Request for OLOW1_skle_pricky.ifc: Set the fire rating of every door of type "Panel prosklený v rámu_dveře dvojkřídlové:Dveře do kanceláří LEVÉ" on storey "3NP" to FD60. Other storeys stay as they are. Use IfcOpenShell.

First a look at what the model holds.

```python
import ifcopenshell
import ifcopenshell.util.element

model = ifcopenshell.open("OLOW1_skle_pricky.ifc")
print(model.schema)
storey = next(s for s in model.by_type("IfcBuildingStorey") if s.Name == "3NP")
doors = [e for e in ifcopenshell.util.element.get_decomposition(storey) if e.is_a("IfcDoor")]
seen = {}
for e in doors:
    element_type = ifcopenshell.util.element.get_type(e)
    key = (element_type.Name if element_type != e and element_type else None, ifcopenshell.util.element.get_pset(e, "Pset_DoorCommon", "FireRating"))
    seen[key] = seen.get(key, 0) + 1
for (name, value), count in sorted(seen.items(), key=str):
    print(count, "x", name, "|", value)
```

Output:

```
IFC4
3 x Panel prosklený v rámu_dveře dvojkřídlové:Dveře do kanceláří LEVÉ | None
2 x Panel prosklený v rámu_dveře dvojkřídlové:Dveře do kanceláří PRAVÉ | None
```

```python
import ifcopenshell
import ifcopenshell.api.pset
import ifcopenshell.util.element

model = ifcopenshell.open("OLOW1_skle_pricky.ifc")

storey = next(s for s in model.by_type("IfcBuildingStorey") if s.Name == "3NP")
doors = [e for e in ifcopenshell.util.element.get_decomposition(storey) if e.is_a("IfcDoor")]

count = 0
for e in doors:
    element_type = ifcopenshell.util.element.get_type(e)
    if element_type in (None, e) or element_type.Name != "Panel prosklený v rámu_dveře dvojkřídlové:Dveře do kanceláří LEVÉ":
        continue
    # add_pset returns the element's existing set when there is one.
    pset = ifcopenshell.api.pset.add_pset(model, product=e, name="Pset_DoorCommon")
    ifcopenshell.api.pset.edit_pset(model, pset=pset, properties={"FireRating": "FD60"})
    count += 1

print(count, "doors updated")

model.write("OLOW1_skle_pricky_rev.ifc")
```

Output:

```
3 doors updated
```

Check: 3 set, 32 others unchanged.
